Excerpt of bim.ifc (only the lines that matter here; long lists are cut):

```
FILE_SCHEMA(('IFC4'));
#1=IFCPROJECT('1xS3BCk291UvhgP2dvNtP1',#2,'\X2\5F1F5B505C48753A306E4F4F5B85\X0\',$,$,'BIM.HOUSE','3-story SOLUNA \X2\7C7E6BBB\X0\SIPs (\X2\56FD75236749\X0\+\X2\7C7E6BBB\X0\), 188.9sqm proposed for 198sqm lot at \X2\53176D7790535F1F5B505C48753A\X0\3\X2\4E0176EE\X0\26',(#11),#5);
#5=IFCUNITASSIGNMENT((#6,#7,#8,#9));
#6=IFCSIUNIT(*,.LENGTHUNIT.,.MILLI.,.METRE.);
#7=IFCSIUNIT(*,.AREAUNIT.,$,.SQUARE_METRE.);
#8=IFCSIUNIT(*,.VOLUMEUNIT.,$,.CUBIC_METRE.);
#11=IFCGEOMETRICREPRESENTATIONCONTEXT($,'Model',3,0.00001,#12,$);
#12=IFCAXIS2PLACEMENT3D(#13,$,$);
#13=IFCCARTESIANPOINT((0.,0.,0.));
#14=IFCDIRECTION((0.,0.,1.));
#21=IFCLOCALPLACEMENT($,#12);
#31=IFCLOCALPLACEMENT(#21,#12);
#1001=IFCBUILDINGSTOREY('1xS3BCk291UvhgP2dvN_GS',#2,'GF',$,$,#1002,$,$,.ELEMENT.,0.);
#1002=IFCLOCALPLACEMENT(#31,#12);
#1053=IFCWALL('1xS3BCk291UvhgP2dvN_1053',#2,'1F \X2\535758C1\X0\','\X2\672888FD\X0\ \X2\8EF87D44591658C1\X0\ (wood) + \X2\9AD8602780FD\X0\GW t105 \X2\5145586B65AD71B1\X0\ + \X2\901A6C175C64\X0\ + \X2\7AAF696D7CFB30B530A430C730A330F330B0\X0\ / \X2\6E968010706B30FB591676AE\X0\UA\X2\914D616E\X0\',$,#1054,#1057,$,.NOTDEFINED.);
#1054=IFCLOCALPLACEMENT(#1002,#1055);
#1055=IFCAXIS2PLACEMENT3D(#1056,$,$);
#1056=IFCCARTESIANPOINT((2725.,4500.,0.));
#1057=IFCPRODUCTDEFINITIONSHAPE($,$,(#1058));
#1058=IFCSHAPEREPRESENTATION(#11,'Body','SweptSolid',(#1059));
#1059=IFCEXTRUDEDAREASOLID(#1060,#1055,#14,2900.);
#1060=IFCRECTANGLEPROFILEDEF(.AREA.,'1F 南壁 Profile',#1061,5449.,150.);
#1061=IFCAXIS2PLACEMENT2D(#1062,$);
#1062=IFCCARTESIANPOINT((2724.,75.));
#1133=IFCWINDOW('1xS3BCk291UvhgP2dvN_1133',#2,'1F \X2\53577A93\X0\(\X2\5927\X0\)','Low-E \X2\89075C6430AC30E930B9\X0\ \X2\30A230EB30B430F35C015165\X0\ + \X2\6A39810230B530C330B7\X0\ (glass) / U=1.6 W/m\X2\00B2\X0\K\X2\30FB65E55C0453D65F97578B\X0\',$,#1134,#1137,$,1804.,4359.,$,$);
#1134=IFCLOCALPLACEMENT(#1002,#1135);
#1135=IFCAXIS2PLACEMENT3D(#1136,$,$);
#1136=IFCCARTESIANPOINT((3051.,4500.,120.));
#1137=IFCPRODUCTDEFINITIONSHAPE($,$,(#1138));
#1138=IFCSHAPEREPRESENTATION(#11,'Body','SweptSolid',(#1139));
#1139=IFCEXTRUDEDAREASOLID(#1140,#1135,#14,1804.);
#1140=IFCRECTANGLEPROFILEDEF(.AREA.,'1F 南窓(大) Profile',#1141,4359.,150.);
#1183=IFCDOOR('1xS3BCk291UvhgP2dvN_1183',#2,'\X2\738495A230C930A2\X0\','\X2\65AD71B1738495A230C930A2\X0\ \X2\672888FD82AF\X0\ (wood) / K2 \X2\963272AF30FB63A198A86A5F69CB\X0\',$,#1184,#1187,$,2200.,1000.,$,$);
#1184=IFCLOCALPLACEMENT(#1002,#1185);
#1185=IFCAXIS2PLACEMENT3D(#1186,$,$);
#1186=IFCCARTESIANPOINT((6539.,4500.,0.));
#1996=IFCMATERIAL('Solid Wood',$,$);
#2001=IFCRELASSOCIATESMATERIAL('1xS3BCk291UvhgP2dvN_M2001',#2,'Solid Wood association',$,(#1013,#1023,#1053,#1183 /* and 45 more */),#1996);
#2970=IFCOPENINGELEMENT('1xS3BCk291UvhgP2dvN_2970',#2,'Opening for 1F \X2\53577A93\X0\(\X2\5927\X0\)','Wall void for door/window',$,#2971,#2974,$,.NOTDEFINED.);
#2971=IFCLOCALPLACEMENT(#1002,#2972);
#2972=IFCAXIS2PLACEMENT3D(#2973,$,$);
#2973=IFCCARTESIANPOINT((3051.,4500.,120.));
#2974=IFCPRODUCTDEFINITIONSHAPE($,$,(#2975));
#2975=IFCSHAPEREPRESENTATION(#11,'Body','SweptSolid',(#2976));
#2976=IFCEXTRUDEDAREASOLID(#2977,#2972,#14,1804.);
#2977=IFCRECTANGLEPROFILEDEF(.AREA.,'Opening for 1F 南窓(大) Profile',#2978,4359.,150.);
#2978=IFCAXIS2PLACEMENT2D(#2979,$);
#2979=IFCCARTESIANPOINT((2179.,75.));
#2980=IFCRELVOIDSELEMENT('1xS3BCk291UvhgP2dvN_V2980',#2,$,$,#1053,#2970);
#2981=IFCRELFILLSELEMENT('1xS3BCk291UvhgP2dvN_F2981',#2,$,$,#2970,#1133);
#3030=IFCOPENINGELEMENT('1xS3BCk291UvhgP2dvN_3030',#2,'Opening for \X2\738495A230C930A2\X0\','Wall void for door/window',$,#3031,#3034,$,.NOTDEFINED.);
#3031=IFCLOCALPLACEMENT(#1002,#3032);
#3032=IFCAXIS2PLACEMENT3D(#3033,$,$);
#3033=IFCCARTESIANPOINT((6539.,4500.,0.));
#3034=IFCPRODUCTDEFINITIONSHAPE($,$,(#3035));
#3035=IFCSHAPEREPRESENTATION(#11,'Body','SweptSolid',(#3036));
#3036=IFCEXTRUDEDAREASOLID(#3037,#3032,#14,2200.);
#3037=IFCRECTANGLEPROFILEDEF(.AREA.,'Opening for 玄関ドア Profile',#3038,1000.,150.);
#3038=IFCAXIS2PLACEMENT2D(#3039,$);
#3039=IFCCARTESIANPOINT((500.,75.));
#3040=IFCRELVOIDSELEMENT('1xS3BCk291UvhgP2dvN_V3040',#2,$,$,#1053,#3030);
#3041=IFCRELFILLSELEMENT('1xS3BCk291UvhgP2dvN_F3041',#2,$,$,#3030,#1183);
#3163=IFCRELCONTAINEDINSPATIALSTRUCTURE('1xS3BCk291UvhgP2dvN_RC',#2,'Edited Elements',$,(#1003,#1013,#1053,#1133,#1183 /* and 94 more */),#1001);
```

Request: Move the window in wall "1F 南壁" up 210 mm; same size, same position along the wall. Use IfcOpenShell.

```python
import numpy as np
import ifcopenshell
import ifcopenshell.api.geometry
import ifcopenshell.util.placement
import ifcopenshell.util.unit

model = ifcopenshell.open("bim.ifc")
unit_scale = ifcopenshell.util.unit.calculate_unit_scale(model)

window = model.by_guid("1xS3BCk291UvhgP2dvN_1133")
opening = window.FillsVoids[0].RelatingOpeningElement
dz = 0.21 / unit_scale

shift = np.array([0.0, 0.0, dz])
# The window is not placed relative to its opening, so move both.
for product in (opening, window):
    matrix = ifcopenshell.util.placement.get_local_placement(product.ObjectPlacement)
    matrix[:3, 3] += shift
    ifcopenshell.api.geometry.edit_object_placement(model, product=product, matrix=matrix, is_si=False)

print(f"moved by {dz * unit_scale:+.3f} m")

model.write("bim_rev.ifc")
```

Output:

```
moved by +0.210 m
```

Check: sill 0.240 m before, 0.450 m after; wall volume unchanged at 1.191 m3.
